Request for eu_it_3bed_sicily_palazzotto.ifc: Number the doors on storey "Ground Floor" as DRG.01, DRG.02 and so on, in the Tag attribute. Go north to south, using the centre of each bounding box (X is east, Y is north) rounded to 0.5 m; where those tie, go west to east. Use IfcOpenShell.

First a look at what the model holds.

```python
import ifcopenshell
import ifcopenshell.util.element
import ifcopenshell.util.placement

model = ifcopenshell.open("eu_it_3bed_sicily_palazzotto.ifc")
print(model.schema)
storey = next(s for s in model.by_type("IfcBuildingStorey") if s.Name == "Ground Floor")
doors = [e for e in ifcopenshell.util.element.get_decomposition(storey) if e.is_a("IfcDoor")]
for e in sorted(doors, key=lambda e: e.id()):
    origin = ifcopenshell.util.placement.get_local_placement(e.ObjectPlacement)[:3, 3]
    print(e.id(), e.Tag, e.Name, origin.round(2) + 0.0, sep=" | ")
```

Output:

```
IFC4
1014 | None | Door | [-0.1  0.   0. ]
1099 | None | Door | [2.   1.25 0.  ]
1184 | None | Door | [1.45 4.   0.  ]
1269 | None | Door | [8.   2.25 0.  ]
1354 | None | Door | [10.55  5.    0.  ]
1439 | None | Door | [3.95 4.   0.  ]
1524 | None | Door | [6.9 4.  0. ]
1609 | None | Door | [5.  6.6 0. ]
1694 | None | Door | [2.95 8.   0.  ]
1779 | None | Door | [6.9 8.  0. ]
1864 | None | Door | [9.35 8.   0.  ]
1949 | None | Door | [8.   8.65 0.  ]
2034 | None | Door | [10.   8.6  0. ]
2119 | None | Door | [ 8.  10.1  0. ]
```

```python
import ifcopenshell
import ifcopenshell.geom
import ifcopenshell.util.element
import ifcopenshell.util.shape

model = ifcopenshell.open("eu_it_3bed_sicily_palazzotto.ifc")
settings = ifcopenshell.geom.settings()
settings.set("use-world-coords", True)


def centre(element):
    shape = ifcopenshell.geom.create_shape(settings, element)
    return ifcopenshell.util.shape.get_bbox_centroid(shape.geometry)


storey = next(s for s in model.by_type("IfcBuildingStorey") if s.Name == "Ground Floor")
doors = [e for e in ifcopenshell.util.element.get_decomposition(storey) if e.is_a("IfcDoor")]

# Insertion points can sit at a corner or the storey origin, so sort by the geometry (in metres).
centres = {e: centre(e) for e in doors}
doors.sort(key=lambda e: (-round(centres[e][1] / 0.5), centres[e][0]))

for i, e in enumerate(doors, start=1):
    number = f"DRG.{i:02d}"
    e.Tag = number
    print(e.id(), number)

model.write("eu_it_3bed_sicily_palazzotto-out.ifc")
```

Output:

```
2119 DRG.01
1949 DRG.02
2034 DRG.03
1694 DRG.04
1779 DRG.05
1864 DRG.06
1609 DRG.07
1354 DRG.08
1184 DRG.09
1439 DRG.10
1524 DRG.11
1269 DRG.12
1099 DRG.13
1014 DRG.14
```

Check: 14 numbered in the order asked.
